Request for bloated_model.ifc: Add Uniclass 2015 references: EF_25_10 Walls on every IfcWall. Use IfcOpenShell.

First a look at what the model holds.

```python
import ifcopenshell

model = ifcopenshell.open("bloated_model.ifc")
print(model.schema)
print("classifications:", [c.Name for c in model.by_type("IfcClassification")])
for ifc_class in ("IfcDoor", "IfcRoof", "IfcStair", "IfcWall", "IfcWindow"):
    print(ifc_class, len(model.by_type(ifc_class)))
```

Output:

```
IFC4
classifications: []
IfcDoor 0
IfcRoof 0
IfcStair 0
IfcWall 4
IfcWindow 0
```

```python
import ifcopenshell
import ifcopenshell.api.classification

model = ifcopenshell.open("bloated_model.ifc")

system = ifcopenshell.api.classification.add_classification(model, classification="Uniclass 2015")

codes = {
    "IfcWall": ("EF_25_10", "Walls"),
}
for ifc_class, (code, name) in codes.items():
    products = model.by_type(ifc_class)
    ifcopenshell.api.classification.add_reference(
        model, products=products, classification=system, identification=code, name=name
    )
    print(code, len(products))

model.write("bloated_model_v2.ifc")
```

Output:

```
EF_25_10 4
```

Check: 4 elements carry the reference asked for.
